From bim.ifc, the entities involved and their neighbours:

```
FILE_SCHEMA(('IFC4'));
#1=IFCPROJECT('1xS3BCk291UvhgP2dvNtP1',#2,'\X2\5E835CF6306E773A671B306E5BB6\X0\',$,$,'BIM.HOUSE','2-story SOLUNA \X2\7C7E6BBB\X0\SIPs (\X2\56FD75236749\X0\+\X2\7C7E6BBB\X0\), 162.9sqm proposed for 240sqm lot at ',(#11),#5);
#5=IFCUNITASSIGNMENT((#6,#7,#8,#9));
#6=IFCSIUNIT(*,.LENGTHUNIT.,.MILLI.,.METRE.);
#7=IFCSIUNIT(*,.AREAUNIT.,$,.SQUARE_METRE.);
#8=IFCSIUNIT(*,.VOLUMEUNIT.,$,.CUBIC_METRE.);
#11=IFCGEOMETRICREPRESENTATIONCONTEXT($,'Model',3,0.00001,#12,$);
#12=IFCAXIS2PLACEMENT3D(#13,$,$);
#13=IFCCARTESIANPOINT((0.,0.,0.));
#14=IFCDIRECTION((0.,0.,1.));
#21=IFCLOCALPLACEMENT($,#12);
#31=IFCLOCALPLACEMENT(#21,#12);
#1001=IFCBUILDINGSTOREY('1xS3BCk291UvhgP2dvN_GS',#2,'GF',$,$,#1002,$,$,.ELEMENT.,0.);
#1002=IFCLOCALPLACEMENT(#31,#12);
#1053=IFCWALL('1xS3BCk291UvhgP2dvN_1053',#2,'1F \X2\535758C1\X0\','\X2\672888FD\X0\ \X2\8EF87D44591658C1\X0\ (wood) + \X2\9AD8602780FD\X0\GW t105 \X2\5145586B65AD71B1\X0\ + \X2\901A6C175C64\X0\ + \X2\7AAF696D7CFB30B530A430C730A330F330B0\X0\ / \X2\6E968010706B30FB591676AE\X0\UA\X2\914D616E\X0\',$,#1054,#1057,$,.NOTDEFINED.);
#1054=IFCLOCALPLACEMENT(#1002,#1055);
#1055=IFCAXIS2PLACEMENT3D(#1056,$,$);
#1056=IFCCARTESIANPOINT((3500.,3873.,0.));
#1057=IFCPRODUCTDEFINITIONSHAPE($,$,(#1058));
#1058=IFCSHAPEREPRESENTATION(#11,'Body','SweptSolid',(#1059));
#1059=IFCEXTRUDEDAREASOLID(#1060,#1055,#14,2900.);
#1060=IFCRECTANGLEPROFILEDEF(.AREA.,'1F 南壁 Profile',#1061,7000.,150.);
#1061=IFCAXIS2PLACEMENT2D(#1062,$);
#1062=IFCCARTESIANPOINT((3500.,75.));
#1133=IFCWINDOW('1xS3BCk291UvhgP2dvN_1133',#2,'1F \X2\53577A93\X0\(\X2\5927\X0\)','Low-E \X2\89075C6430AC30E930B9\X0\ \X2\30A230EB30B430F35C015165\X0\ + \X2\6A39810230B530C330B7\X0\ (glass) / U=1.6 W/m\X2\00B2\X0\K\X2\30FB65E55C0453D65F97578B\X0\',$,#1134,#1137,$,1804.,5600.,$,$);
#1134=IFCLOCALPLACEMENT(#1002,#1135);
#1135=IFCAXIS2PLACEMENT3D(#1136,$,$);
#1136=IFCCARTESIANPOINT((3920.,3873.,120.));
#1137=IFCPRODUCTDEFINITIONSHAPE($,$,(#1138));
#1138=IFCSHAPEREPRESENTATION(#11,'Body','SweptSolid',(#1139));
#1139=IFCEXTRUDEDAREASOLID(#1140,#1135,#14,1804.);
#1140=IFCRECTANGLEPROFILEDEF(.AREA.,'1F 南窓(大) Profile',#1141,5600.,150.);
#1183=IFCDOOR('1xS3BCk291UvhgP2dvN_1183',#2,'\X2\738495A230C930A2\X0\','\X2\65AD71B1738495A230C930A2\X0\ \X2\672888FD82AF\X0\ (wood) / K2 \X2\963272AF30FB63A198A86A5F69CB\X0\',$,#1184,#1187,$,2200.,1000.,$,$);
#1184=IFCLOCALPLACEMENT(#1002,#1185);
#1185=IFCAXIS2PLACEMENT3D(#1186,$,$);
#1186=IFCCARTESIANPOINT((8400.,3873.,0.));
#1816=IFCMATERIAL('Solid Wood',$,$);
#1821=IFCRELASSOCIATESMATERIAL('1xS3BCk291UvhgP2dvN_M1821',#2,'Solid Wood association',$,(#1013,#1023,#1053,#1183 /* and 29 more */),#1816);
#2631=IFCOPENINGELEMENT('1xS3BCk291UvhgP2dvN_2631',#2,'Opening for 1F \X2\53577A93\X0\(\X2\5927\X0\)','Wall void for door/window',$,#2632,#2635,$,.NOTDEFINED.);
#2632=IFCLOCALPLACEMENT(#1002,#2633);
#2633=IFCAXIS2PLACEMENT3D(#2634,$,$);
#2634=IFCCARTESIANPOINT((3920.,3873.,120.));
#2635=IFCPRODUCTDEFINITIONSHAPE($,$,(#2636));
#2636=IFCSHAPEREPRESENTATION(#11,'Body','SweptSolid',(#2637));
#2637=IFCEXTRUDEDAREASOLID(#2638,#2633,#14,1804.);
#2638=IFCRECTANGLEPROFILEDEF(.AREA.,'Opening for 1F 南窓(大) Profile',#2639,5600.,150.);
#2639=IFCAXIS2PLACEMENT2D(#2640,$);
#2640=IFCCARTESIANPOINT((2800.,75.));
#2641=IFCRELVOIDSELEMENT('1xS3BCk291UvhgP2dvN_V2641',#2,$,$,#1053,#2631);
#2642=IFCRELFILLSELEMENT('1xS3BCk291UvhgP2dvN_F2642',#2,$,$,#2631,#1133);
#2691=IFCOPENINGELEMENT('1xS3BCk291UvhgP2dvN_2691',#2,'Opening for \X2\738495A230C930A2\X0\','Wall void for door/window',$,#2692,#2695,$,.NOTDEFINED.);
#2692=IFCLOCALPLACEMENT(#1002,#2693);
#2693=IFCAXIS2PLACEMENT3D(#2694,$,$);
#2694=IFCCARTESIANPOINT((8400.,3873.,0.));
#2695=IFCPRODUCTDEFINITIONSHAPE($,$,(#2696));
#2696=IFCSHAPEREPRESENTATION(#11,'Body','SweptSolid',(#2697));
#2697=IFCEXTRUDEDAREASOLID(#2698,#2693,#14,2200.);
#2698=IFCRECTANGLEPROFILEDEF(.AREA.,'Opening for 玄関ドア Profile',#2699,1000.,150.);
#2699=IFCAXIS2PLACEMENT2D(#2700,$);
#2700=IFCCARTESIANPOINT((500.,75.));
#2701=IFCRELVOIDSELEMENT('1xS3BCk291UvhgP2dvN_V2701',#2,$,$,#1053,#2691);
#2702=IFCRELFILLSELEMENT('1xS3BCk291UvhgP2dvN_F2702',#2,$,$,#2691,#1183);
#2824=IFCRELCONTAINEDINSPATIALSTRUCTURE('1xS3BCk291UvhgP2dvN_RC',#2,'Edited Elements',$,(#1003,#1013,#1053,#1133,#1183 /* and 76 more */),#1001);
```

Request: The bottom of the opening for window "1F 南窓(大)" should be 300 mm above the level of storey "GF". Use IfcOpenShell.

```python
import numpy as np
import ifcopenshell
import ifcopenshell.api.geometry
import ifcopenshell.geom
import ifcopenshell.util.element
import ifcopenshell.util.placement
import ifcopenshell.util.shape
import ifcopenshell.util.unit

model = ifcopenshell.open("bim.ifc")
unit_scale = ifcopenshell.util.unit.calculate_unit_scale(model)

window = model.by_id(1133)
opening = window.FillsVoids[0].RelatingOpeningElement
storey = ifcopenshell.util.element.get_container(window, ifc_class="IfcBuildingStorey")
level = ifcopenshell.util.placement.get_local_placement(storey.ObjectPlacement)[2, 3]

# The opening's origin need not be at the sill, so measure its lowest point.
shape = ifcopenshell.geom.create_shape(ifcopenshell.geom.settings(), opening)
bottom = ifcopenshell.util.shape.get_shape_bottom_elevation(shape, shape.geometry) / unit_scale
dz = level + 0.3 / unit_scale - bottom

shift = np.array([0.0, 0.0, dz])
# The window is not placed relative to its opening, so move both.
for product in (opening, window):
    matrix = ifcopenshell.util.placement.get_local_placement(product.ObjectPlacement)
    matrix[:3, 3] += shift
    ifcopenshell.api.geometry.edit_object_placement(model, product=product, matrix=matrix, is_si=False)

print(f"moved by {dz * unit_scale:+.3f} m")

model.write("bim_rev.ifc")
```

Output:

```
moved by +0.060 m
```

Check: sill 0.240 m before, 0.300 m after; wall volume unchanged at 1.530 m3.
